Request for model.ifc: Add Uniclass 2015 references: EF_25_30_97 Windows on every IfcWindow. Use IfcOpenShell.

First a look at what the model holds.

```python
import ifcopenshell

model = ifcopenshell.open("model.ifc")
print(model.schema)
print("classifications:", [c.Name for c in model.by_type("IfcClassification")])
for ifc_class in ("IfcDoor", "IfcRoof", "IfcStair", "IfcWall", "IfcWindow"):
    print(ifc_class, len(model.by_type(ifc_class)))
```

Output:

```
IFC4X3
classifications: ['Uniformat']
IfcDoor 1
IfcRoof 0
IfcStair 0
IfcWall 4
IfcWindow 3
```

```python
import ifcopenshell
import ifcopenshell.api.classification

model = ifcopenshell.open("model.ifc")

system = ifcopenshell.api.classification.add_classification(model, classification="Uniclass 2015")

codes = {
    "IfcWindow": ("EF_25_30_97", "Windows"),
}
for ifc_class, (code, name) in codes.items():
    products = model.by_type(ifc_class)
    ifcopenshell.api.classification.add_reference(
        model, products=products, classification=system, identification=code, name=name
    )
    print(code, len(products))

model.write("model_updated.ifc")
```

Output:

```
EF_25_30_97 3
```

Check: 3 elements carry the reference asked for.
